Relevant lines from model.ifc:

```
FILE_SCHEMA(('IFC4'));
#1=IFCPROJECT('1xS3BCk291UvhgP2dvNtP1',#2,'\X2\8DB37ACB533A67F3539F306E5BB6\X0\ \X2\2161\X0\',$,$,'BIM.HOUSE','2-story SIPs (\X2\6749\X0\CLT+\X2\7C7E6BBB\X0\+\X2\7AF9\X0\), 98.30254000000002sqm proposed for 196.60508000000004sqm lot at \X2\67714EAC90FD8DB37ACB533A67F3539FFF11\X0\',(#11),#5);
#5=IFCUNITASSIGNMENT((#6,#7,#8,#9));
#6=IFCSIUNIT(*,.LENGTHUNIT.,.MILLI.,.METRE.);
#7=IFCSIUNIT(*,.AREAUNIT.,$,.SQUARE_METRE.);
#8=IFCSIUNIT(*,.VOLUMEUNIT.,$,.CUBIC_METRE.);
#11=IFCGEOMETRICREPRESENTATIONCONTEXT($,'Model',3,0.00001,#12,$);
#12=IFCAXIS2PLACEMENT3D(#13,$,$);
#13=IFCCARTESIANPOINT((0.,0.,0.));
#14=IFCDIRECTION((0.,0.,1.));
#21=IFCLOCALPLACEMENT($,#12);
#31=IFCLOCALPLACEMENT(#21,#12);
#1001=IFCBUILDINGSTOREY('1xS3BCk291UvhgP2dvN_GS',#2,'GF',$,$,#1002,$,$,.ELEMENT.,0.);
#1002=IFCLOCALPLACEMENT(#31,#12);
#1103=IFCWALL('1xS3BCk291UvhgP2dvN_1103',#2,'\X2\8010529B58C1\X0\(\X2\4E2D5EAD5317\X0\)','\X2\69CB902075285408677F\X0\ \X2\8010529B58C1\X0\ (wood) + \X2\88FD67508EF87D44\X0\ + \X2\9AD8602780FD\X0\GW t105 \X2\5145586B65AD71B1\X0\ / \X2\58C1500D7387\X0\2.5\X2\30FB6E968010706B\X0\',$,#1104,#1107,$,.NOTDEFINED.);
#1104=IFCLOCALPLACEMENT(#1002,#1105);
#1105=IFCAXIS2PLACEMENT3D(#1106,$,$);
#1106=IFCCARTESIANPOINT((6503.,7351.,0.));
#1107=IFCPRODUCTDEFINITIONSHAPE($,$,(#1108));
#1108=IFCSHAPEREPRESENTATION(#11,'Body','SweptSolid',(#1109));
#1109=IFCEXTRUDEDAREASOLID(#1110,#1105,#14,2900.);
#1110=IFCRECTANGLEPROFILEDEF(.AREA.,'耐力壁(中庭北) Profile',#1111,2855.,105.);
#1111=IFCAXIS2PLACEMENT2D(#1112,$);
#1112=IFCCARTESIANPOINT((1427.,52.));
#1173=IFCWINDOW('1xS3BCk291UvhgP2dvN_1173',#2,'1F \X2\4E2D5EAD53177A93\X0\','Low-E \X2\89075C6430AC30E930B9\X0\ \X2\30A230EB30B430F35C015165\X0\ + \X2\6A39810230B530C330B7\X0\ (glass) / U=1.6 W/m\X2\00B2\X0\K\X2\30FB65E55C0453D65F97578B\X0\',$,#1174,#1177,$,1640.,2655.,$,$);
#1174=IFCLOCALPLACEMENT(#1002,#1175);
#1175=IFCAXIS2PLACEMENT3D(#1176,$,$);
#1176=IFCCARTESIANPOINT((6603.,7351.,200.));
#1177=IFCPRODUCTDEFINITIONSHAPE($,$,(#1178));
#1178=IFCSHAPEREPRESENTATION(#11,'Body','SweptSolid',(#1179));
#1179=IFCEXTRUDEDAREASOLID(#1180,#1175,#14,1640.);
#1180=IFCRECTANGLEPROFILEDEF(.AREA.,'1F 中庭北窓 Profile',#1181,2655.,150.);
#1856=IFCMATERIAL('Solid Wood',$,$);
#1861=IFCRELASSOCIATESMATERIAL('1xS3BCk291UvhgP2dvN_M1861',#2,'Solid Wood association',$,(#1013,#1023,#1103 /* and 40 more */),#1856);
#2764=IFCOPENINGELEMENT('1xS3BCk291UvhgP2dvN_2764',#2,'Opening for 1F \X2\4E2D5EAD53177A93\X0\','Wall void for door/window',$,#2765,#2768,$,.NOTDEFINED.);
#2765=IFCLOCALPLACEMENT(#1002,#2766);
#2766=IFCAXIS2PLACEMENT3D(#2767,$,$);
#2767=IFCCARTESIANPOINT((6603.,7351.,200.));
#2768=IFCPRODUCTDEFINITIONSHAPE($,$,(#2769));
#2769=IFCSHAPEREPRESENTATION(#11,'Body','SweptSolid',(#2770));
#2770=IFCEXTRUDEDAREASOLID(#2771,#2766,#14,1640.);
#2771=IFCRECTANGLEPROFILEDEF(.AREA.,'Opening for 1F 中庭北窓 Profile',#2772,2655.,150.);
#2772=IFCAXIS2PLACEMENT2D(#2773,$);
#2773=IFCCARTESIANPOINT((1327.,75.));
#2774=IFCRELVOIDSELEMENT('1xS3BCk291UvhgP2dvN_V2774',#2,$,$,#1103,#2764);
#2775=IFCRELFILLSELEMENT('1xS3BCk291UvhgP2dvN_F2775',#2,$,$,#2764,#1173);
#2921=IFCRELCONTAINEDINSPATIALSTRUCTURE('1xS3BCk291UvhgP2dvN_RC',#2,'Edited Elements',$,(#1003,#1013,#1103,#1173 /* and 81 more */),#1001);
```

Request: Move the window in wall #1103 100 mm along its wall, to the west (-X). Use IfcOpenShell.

```python
import ifcopenshell
import ifcopenshell.api.geometry
import ifcopenshell.util.placement

model = ifcopenshell.open("model.ifc")

window = model.by_guid("1xS3BCk291UvhgP2dvN_1173")
opening = window.FillsVoids[0].RelatingOpeningElement
wall = opening.VoidsElements[0].RelatingBuildingElement

wall_matrix = ifcopenshell.util.placement.get_local_placement(wall.ObjectPlacement)
shift = wall_matrix[:3, 0] * -100.0
before = ifcopenshell.util.placement.get_local_placement(window.ObjectPlacement)[:3, 3].copy()

# The window is not placed relative to its opening, so move both.
for product in (opening, window):
    matrix = ifcopenshell.util.placement.get_local_placement(product.ObjectPlacement)
    matrix[:3, 3] += shift
    ifcopenshell.api.geometry.edit_object_placement(model, product=product, matrix=matrix, is_si=False)

after = ifcopenshell.util.placement.get_local_placement(window.ObjectPlacement)[:3, 3]
print("window moved by", (after - before).round(3) + 0.0)

model.write("model_v2.ifc")
```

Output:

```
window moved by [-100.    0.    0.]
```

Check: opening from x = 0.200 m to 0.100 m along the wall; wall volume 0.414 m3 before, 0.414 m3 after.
